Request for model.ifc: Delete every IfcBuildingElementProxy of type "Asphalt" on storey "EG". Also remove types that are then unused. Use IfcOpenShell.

First a look at what the model holds.

```python
import ifcopenshell
import ifcopenshell.util.element

model = ifcopenshell.open("model.ifc")
print(model.schema)
storey = next(s for s in model.by_type("IfcBuildingStorey") if s.Name == "EG")
proxies = [e for e in ifcopenshell.util.element.get_decomposition(storey) if e.is_a("IfcBuildingElementProxy")]
seen = {}
for e in proxies:
    element_type = ifcopenshell.util.element.get_type(e)
    name = element_type.Name if element_type not in (None, e) else None
    seen[name] = seen.get(name, 0) + 1
for name, count in sorted(seen.items(), key=str):
    print(count, "x", name)
```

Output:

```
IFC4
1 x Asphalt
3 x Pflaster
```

```python
import ifcopenshell
import ifcopenshell.api.root
import ifcopenshell.util.element

model = ifcopenshell.open("model.ifc")

storey = next(s for s in model.by_type("IfcBuildingStorey") if s.Name == "EG")
proxies = [e for e in ifcopenshell.util.element.get_decomposition(storey) if e.is_a("IfcBuildingElementProxy")]
targets = [e for e in proxies if (t := ifcopenshell.util.element.get_type(e)) not in (None, e) and t.Name == "Asphalt"]
types = {ifcopenshell.util.element.get_type(e) for e in targets} - {None, *targets}

for e in targets:
    ifcopenshell.api.root.remove_product(model, product=e)
print(len(targets), "removed")

unused = [t for t in types if not ifcopenshell.util.element.get_types(t)]
for t in unused:
    ifcopenshell.api.root.remove_product(model, product=t)
print(len(unused), "unused types removed")

model.write("model_rev.ifc")
```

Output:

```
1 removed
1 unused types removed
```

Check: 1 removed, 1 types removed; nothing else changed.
